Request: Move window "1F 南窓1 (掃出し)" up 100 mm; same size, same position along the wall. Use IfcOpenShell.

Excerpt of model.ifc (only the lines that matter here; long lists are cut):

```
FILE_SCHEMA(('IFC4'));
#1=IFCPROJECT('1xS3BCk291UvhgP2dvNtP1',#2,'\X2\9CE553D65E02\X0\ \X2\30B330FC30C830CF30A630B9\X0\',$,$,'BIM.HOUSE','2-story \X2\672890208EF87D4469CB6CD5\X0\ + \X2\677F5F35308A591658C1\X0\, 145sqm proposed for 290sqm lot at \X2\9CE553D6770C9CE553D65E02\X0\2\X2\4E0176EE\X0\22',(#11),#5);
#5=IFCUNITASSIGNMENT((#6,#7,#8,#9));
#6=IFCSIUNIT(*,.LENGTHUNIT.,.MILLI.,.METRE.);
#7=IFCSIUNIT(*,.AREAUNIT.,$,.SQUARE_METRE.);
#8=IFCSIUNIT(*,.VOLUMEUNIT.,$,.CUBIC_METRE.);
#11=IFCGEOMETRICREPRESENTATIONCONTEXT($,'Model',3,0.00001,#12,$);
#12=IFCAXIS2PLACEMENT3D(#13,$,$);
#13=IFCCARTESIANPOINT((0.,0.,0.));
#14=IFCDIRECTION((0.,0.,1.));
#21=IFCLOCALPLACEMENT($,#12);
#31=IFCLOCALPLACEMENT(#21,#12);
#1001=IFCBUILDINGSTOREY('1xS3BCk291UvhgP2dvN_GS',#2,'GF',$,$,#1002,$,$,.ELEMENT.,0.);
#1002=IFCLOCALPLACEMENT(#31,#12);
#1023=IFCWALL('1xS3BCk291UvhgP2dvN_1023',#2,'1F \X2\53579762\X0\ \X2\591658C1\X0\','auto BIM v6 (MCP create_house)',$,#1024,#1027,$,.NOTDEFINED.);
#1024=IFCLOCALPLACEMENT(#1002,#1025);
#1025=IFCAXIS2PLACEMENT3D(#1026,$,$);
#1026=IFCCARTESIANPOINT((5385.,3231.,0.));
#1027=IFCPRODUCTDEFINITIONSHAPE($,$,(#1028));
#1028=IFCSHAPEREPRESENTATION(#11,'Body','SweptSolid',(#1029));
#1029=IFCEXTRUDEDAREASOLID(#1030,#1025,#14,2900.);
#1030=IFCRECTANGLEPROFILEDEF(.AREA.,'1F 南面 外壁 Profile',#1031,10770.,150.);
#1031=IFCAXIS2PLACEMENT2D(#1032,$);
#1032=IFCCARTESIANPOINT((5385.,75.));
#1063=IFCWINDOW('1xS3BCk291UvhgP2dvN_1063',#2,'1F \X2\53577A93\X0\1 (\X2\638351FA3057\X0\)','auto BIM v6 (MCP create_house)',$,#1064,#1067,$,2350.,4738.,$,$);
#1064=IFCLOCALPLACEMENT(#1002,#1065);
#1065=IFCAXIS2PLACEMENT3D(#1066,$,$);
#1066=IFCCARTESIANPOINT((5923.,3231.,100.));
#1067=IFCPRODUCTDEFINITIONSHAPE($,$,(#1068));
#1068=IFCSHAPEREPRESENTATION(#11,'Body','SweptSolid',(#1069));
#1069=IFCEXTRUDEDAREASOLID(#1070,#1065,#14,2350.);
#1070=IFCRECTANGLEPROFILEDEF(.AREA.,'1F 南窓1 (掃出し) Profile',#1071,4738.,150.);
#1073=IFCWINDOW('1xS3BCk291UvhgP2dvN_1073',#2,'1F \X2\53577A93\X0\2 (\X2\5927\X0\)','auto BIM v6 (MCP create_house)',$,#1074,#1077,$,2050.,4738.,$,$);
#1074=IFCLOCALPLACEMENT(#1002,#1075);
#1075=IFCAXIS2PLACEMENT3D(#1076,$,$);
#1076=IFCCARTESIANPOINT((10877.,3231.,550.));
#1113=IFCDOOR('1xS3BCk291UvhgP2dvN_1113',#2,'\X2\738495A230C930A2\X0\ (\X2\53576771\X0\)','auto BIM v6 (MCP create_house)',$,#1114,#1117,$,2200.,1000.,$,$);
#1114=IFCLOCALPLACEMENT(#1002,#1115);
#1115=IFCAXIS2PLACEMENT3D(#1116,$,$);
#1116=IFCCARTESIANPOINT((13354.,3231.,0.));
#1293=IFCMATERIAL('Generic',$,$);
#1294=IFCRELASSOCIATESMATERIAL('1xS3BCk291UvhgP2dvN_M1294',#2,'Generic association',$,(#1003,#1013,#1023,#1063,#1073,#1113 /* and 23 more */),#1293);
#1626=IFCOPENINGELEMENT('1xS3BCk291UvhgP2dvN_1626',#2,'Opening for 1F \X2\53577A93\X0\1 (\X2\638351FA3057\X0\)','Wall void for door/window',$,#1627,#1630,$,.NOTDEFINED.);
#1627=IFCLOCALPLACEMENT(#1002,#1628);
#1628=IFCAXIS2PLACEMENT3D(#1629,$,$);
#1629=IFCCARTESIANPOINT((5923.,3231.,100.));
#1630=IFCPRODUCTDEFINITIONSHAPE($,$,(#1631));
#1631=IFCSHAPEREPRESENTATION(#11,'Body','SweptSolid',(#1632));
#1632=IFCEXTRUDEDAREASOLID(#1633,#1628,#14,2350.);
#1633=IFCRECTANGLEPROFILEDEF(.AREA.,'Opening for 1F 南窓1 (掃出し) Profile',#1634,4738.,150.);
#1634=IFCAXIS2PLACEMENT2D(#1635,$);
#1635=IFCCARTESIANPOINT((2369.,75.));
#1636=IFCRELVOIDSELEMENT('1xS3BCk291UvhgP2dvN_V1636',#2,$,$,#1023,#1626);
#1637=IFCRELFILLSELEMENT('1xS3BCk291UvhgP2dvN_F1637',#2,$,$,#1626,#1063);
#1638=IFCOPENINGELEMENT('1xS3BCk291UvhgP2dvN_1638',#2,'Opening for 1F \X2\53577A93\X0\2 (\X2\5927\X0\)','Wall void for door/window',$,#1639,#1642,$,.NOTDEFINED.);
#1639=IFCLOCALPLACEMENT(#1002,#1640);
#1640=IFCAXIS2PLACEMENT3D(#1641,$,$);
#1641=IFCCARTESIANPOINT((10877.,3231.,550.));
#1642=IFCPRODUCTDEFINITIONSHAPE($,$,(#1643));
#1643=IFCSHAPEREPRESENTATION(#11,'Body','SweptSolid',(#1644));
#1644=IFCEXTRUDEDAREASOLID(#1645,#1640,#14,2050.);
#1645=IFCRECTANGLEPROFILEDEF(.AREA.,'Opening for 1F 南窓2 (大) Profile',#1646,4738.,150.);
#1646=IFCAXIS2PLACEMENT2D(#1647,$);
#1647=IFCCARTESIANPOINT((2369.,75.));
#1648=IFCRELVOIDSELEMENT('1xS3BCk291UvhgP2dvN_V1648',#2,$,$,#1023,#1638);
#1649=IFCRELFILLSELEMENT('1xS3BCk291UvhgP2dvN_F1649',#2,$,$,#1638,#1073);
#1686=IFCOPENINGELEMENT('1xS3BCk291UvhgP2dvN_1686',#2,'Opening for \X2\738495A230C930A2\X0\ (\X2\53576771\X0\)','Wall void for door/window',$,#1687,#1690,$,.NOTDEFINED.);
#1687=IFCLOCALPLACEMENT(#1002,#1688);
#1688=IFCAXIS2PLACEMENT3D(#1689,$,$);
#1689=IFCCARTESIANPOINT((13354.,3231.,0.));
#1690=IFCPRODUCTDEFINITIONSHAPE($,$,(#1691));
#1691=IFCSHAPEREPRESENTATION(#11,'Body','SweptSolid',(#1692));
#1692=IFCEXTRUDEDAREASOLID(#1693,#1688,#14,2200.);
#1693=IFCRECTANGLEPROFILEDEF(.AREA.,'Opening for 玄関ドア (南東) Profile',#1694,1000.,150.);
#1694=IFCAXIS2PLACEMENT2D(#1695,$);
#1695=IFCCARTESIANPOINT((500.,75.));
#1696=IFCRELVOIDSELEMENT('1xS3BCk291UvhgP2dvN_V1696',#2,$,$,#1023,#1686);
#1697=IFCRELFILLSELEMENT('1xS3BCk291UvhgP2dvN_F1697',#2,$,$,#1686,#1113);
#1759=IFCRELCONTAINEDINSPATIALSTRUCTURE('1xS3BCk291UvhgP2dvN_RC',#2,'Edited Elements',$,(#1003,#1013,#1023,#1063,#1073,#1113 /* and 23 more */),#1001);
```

```python
import numpy as np
import ifcopenshell
import ifcopenshell.api.geometry
import ifcopenshell.util.placement
import ifcopenshell.util.unit

model = ifcopenshell.open("model.ifc")
unit_scale = ifcopenshell.util.unit.calculate_unit_scale(model)

window = model.by_id(1063)
opening = window.FillsVoids[0].RelatingOpeningElement
dz = 100.0

shift = np.array([0.0, 0.0, dz])
# The window is not placed relative to its opening, so move both.
for product in (opening, window):
    matrix = ifcopenshell.util.placement.get_local_placement(product.ObjectPlacement)
    matrix[:3, 3] += shift
    ifcopenshell.api.geometry.edit_object_placement(model, product=product, matrix=matrix, is_si=False)

print(f"moved by {dz * unit_scale:+.3f} m")

model.write("model_edited.ifc")
```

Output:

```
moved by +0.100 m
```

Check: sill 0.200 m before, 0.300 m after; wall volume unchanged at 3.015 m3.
